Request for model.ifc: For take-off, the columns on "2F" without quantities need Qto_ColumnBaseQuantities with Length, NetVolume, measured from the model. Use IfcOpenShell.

First a look at what the model holds.

```python
import ifcopenshell
import ifcopenshell.util.element
import ifcopenshell.util.unit

model = ifcopenshell.open("model.ifc")
print(model.schema)
for unit_type in ("LENGTHUNIT", "AREAUNIT", "VOLUMEUNIT"):
    print(unit_type, ifcopenshell.util.unit.calculate_unit_scale(model, unit_type))
storey = next(s for s in model.by_type("IfcBuildingStorey") if s.Name == "2F")
columns = [e for e in ifcopenshell.util.element.get_decomposition(storey) if e.is_a("IfcColumn")]
for e in sorted(columns, key=lambda e: e.id()):
    print(e.id(), e.is_a(), e.Name, list(ifcopenshell.util.element.get_psets(e, qtos_only=True)), sep=" | ")
```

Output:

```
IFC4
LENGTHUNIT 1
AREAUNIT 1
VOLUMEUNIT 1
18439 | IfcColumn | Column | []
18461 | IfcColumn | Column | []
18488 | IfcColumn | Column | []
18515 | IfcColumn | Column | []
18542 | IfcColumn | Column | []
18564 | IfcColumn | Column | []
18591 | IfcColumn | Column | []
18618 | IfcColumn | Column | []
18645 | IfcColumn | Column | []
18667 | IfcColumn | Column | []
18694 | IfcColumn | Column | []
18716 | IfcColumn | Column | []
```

```python
import ifcopenshell
import ifcopenshell.api.pset
import ifcopenshell.geom
import ifcopenshell.util.element
import ifcopenshell.util.shape
import ifcopenshell.util.unit

model = ifcopenshell.open("model.ifc")
unit_scale = ifcopenshell.util.unit.calculate_unit_scale(model)
volume_scale = ifcopenshell.util.unit.calculate_unit_scale(model, "VOLUMEUNIT")
settings = ifcopenshell.geom.settings()

storey = next(s for s in model.by_type("IfcBuildingStorey") if s.Name == "2F")
columns = [e for e in ifcopenshell.util.element.get_decomposition(storey) if e.is_a("IfcColumn")]

for e in sorted(columns, key=lambda e: e.id()):
    if ifcopenshell.util.element.get_psets(e, qtos_only=True, should_inherit=False):
        continue
    # Geometry comes back in metres, in the element's own axes.
    shape = ifcopenshell.geom.create_shape(settings, e)
    values = {
        "Length": ifcopenshell.util.shape.get_z(shape.geometry) / unit_scale,
        "NetVolume": ifcopenshell.util.shape.get_volume(shape.geometry) / volume_scale,
    }
    qto = ifcopenshell.api.pset.add_qto(model, product=e, name="Qto_ColumnBaseQuantities")
    ifcopenshell.api.pset.edit_qto(model, qto=qto, properties=values)
    print(e.id(), {k: round(v, 3) for k, v in values.items()})

model.write("model_rev.ifc")
```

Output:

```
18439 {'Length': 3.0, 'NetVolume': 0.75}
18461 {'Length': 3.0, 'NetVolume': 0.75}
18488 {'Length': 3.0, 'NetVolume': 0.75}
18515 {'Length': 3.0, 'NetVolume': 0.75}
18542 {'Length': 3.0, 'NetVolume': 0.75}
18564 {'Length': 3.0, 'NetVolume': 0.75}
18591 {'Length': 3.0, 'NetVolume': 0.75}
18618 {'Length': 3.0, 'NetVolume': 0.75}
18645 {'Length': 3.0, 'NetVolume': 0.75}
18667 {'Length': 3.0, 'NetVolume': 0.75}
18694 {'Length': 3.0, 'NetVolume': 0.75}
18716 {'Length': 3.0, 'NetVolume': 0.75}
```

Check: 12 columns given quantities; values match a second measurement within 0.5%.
